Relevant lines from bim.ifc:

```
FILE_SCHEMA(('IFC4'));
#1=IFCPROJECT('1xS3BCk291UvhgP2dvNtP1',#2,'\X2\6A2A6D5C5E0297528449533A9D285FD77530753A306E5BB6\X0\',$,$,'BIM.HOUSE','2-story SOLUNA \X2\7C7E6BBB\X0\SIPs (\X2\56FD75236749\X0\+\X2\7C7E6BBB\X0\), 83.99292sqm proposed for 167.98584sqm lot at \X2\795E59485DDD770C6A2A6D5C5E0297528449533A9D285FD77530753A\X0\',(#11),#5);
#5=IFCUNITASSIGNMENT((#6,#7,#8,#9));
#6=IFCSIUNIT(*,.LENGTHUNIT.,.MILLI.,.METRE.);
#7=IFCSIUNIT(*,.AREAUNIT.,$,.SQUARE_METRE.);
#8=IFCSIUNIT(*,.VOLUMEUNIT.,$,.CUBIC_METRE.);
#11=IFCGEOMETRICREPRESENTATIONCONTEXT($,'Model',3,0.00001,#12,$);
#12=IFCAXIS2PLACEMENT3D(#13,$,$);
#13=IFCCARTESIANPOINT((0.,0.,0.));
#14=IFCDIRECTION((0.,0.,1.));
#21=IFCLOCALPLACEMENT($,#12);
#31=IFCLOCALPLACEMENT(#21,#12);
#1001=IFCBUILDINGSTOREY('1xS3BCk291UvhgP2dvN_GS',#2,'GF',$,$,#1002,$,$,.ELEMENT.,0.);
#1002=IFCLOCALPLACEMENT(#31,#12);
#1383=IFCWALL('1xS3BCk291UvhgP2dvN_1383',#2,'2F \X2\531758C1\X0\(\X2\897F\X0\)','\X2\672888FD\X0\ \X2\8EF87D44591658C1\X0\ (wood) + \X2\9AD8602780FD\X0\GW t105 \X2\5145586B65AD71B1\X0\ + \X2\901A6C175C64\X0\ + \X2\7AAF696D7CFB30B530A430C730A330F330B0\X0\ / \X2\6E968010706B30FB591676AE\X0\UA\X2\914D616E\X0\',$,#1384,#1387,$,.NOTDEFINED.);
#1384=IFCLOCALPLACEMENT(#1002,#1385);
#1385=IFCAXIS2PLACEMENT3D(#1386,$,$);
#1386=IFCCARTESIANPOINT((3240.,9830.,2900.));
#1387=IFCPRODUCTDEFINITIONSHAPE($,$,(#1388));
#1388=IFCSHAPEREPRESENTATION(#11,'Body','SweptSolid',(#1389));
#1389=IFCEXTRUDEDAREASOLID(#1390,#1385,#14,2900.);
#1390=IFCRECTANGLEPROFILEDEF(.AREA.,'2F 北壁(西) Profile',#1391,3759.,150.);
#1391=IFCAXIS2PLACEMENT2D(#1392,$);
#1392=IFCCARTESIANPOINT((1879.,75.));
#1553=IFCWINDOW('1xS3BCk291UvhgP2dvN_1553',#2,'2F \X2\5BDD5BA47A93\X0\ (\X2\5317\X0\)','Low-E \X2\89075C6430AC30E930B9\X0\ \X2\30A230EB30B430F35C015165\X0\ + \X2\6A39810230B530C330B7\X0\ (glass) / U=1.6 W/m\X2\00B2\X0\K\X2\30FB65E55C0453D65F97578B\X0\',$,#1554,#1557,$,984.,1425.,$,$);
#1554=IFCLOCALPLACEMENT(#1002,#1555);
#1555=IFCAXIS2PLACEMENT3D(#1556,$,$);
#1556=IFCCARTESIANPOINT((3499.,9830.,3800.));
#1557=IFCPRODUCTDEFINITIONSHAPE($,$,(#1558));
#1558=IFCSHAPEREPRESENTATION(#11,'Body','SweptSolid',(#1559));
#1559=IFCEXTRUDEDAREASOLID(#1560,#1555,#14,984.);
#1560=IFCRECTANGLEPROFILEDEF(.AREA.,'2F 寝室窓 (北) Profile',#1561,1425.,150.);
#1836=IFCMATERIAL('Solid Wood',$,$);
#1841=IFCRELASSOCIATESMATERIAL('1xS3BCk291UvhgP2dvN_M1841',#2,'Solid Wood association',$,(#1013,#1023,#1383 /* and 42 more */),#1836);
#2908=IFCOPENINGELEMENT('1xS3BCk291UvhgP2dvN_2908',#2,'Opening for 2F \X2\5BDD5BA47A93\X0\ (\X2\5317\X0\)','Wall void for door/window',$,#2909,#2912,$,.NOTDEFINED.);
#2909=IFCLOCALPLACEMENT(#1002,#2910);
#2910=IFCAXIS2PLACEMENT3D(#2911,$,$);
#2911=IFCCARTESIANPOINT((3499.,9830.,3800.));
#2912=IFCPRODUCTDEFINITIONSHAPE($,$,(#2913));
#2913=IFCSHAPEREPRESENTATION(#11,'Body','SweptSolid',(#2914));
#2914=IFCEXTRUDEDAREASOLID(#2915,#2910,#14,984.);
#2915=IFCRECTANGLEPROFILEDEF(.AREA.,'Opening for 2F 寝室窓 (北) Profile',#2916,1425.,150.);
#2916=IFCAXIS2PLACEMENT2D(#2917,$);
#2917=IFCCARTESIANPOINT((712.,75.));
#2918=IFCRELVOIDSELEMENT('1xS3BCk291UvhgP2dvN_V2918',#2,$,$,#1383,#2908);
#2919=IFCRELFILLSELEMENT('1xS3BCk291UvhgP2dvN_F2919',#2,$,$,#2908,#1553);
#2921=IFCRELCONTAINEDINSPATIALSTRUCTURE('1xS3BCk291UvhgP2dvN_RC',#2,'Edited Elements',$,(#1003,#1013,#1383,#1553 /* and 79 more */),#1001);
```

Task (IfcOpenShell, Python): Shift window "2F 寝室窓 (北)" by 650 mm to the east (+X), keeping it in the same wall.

```python
import ifcopenshell
import ifcopenshell.api.geometry
import ifcopenshell.util.placement
import ifcopenshell.util.unit

model = ifcopenshell.open("bim.ifc")
unit_scale = ifcopenshell.util.unit.calculate_unit_scale(model)

window = model.by_id(1553)
opening = window.FillsVoids[0].RelatingOpeningElement
wall = opening.VoidsElements[0].RelatingBuildingElement

wall_matrix = ifcopenshell.util.placement.get_local_placement(wall.ObjectPlacement)
shift = wall_matrix[:3, 0] * 0.65 / unit_scale
before = ifcopenshell.util.placement.get_local_placement(window.ObjectPlacement)[:3, 3].copy()

# The window is not placed relative to its opening, so move both.
for product in (opening, window):
    matrix = ifcopenshell.util.placement.get_local_placement(product.ObjectPlacement)
    matrix[:3, 3] += shift
    ifcopenshell.api.geometry.edit_object_placement(model, product=product, matrix=matrix, is_si=False)

after = ifcopenshell.util.placement.get_local_placement(window.ObjectPlacement)[:3, 3]
print("window moved by", (after - before).round(3) + 0.0)

model.write("bim_v2.ifc")
```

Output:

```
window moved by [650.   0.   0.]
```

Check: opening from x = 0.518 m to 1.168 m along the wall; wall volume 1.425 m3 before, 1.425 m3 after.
